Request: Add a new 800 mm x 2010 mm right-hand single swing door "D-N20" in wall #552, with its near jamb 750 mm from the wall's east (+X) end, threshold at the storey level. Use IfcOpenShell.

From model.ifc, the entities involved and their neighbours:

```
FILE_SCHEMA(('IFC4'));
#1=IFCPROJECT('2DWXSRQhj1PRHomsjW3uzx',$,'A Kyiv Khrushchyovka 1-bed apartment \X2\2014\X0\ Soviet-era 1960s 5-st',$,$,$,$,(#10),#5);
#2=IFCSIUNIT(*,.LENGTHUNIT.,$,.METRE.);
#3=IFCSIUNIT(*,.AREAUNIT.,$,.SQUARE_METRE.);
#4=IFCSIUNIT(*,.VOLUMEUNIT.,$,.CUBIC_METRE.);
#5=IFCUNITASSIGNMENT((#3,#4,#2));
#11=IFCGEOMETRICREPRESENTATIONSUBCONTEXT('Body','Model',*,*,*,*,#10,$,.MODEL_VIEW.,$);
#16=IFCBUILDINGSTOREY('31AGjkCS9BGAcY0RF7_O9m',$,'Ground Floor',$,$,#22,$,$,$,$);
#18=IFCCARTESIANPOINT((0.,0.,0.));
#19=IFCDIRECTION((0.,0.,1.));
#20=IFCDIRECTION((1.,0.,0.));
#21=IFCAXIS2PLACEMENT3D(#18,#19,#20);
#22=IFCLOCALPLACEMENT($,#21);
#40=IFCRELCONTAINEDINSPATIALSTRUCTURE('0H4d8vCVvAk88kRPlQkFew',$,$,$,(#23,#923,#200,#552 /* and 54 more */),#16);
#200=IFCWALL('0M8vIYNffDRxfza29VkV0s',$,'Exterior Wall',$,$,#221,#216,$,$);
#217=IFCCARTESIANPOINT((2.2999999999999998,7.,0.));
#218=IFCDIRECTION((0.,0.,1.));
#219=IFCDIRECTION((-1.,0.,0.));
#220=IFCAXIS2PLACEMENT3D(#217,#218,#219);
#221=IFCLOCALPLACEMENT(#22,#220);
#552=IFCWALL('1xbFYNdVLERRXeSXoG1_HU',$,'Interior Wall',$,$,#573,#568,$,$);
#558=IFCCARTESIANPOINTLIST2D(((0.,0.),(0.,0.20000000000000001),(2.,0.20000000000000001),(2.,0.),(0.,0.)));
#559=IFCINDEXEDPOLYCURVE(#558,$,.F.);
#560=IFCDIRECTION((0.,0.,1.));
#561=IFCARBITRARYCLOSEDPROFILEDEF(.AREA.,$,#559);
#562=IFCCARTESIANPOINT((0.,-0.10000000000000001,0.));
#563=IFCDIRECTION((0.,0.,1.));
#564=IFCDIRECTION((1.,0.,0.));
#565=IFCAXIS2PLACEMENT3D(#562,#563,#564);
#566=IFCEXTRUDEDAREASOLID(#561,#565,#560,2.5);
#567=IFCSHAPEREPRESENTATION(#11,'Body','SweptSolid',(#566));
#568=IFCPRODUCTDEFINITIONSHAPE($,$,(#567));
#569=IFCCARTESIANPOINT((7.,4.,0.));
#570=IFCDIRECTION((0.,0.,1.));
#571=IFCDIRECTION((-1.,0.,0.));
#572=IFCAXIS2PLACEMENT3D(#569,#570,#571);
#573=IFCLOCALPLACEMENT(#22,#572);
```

```python
import numpy as np
import ifcopenshell
import ifcopenshell.api.feature
import ifcopenshell.api.geometry
import ifcopenshell.api.root
import ifcopenshell.api.spatial
import ifcopenshell.geom
import ifcopenshell.util.element
import ifcopenshell.util.placement
import ifcopenshell.util.representation
import ifcopenshell.util.shape
import ifcopenshell.util.unit

model = ifcopenshell.open("model.ifc")
unit_scale = ifcopenshell.util.unit.calculate_unit_scale(model)
settings = ifcopenshell.geom.settings()


def volume(element):
    """Net volume in cubic metres, openings subtracted."""
    shape = ifcopenshell.geom.create_shape(settings, element)
    return ifcopenshell.util.shape.get_volume(shape.geometry)


wall = model.by_guid("1xbFYNdVLERRXeSXoG1_HU")
storey = ifcopenshell.util.element.get_container(wall, ifc_class="IfcBuildingStorey")
context = ifcopenshell.util.representation.get_context(model, "Model", "Body", "MODEL_VIEW")
before = volume(wall)

width, height, from_end, sill = 0.8, 2.01, 0.75, 0.0  # metres

# The wall runs along its own X axis, and the end named is its -X end.
wall_shape = ifcopenshell.geom.create_shape(settings, wall)
x, y, z = ifcopenshell.util.shape.get_vertices(wall_shape.geometry).T
start = x.min() + from_end
face, thickness = float(y.min()), float(y.max() - y.min())
wall_matrix = ifcopenshell.util.placement.get_local_placement(wall.ObjectPlacement)
level = ifcopenshell.util.placement.get_local_placement(storey.ObjectPlacement)[2, 3]


def in_wall(x, y):
    """Placement at x, y metres in the wall's axes, at sill height."""
    matrix = wall_matrix.copy()
    matrix[:, 3] = wall_matrix @ np.array([x / unit_scale, y / unit_scale, 0.0, 1.0])
    matrix[2, 3] = level + sill / unit_scale
    return matrix


# Opening: a box that overshoots both wall faces by 50 mm.
opening = ifcopenshell.api.root.create_entity(model, ifc_class="IfcOpeningElement", predefined_type="OPENING")
box = ifcopenshell.api.geometry.add_wall_representation(
    model, context=context, length=width, height=height, thickness=thickness + 0.1
)
ifcopenshell.api.geometry.assign_representation(model, product=opening, representation=box)
ifcopenshell.api.geometry.edit_object_placement(model, product=opening, matrix=in_wall(start, face - 0.05), is_si=False)
ifcopenshell.api.feature.add_feature(model, feature=opening, element=wall)

door = ifcopenshell.api.root.create_entity(model, ifc_class="IfcDoor", name="D-N20", predefined_type="DOOR")
door.OverallWidth, door.OverallHeight = width / unit_scale, height / unit_scale
door.OperationType = "SINGLE_SWING_RIGHT"
body = ifcopenshell.api.geometry.add_door_representation(
    model,
    context=context,
    overall_width=door.OverallWidth,
    overall_height=door.OverallHeight,
    operation_type="SINGLE_SWING_RIGHT",
    lining_properties={"LiningDepth": thickness / unit_scale, "ThresholdDepth": thickness / unit_scale},
)
ifcopenshell.api.geometry.assign_representation(model, product=door, representation=body)
ifcopenshell.api.spatial.assign_container(model, products=[door], relating_structure=storey)
ifcopenshell.api.feature.add_filling(model, opening=opening, element=door)

# The lining spans the wall, so the door starts at the wall face.
ifcopenshell.api.geometry.edit_object_placement(model, product=door, matrix=in_wall(start, face), is_si=False)

after = volume(wall)

print(f"wall volume {before:.3f} -> {after:.3f} m3")

model.write("model_edited.ifc")
```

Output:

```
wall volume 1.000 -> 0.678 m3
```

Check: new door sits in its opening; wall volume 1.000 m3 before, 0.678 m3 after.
